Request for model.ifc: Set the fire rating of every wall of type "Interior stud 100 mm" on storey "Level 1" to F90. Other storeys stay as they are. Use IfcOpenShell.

First a look at what the model holds.

```python
import ifcopenshell
import ifcopenshell.util.element

model = ifcopenshell.open("model.ifc")
print(model.schema)
storey = next(s for s in model.by_type("IfcBuildingStorey") if s.Name == "Level 1")
walls = [e for e in ifcopenshell.util.element.get_decomposition(storey) if e.is_a("IfcWall")]
seen = {}
for e in walls:
    element_type = ifcopenshell.util.element.get_type(e)
    key = (element_type.Name if element_type != e and element_type else None, ifcopenshell.util.element.get_pset(e, "Pset_WallCommon", "FireRating"))
    seen[key] = seen.get(key, 0) + 1
for (name, value), count in sorted(seen.items(), key=str):
    print(count, "x", name, "|", value)
```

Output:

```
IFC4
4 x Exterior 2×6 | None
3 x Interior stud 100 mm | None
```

```python
import ifcopenshell
import ifcopenshell.api.pset
import ifcopenshell.util.element

model = ifcopenshell.open("model.ifc")

storey = next(s for s in model.by_type("IfcBuildingStorey") if s.Name == "Level 1")
walls = [e for e in ifcopenshell.util.element.get_decomposition(storey) if e.is_a("IfcWall")]

count = 0
for e in walls:
    element_type = ifcopenshell.util.element.get_type(e)
    if element_type in (None, e) or element_type.Name != "Interior stud 100 mm":
        continue
    # add_pset returns the element's existing set when there is one.
    pset = ifcopenshell.api.pset.add_pset(model, product=e, name="Pset_WallCommon")
    ifcopenshell.api.pset.edit_pset(model, pset=pset, properties={"FireRating": "F90"})
    count += 1

print(count, "walls updated")

model.write("model_rev.ifc")
```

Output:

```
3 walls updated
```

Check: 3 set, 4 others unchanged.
